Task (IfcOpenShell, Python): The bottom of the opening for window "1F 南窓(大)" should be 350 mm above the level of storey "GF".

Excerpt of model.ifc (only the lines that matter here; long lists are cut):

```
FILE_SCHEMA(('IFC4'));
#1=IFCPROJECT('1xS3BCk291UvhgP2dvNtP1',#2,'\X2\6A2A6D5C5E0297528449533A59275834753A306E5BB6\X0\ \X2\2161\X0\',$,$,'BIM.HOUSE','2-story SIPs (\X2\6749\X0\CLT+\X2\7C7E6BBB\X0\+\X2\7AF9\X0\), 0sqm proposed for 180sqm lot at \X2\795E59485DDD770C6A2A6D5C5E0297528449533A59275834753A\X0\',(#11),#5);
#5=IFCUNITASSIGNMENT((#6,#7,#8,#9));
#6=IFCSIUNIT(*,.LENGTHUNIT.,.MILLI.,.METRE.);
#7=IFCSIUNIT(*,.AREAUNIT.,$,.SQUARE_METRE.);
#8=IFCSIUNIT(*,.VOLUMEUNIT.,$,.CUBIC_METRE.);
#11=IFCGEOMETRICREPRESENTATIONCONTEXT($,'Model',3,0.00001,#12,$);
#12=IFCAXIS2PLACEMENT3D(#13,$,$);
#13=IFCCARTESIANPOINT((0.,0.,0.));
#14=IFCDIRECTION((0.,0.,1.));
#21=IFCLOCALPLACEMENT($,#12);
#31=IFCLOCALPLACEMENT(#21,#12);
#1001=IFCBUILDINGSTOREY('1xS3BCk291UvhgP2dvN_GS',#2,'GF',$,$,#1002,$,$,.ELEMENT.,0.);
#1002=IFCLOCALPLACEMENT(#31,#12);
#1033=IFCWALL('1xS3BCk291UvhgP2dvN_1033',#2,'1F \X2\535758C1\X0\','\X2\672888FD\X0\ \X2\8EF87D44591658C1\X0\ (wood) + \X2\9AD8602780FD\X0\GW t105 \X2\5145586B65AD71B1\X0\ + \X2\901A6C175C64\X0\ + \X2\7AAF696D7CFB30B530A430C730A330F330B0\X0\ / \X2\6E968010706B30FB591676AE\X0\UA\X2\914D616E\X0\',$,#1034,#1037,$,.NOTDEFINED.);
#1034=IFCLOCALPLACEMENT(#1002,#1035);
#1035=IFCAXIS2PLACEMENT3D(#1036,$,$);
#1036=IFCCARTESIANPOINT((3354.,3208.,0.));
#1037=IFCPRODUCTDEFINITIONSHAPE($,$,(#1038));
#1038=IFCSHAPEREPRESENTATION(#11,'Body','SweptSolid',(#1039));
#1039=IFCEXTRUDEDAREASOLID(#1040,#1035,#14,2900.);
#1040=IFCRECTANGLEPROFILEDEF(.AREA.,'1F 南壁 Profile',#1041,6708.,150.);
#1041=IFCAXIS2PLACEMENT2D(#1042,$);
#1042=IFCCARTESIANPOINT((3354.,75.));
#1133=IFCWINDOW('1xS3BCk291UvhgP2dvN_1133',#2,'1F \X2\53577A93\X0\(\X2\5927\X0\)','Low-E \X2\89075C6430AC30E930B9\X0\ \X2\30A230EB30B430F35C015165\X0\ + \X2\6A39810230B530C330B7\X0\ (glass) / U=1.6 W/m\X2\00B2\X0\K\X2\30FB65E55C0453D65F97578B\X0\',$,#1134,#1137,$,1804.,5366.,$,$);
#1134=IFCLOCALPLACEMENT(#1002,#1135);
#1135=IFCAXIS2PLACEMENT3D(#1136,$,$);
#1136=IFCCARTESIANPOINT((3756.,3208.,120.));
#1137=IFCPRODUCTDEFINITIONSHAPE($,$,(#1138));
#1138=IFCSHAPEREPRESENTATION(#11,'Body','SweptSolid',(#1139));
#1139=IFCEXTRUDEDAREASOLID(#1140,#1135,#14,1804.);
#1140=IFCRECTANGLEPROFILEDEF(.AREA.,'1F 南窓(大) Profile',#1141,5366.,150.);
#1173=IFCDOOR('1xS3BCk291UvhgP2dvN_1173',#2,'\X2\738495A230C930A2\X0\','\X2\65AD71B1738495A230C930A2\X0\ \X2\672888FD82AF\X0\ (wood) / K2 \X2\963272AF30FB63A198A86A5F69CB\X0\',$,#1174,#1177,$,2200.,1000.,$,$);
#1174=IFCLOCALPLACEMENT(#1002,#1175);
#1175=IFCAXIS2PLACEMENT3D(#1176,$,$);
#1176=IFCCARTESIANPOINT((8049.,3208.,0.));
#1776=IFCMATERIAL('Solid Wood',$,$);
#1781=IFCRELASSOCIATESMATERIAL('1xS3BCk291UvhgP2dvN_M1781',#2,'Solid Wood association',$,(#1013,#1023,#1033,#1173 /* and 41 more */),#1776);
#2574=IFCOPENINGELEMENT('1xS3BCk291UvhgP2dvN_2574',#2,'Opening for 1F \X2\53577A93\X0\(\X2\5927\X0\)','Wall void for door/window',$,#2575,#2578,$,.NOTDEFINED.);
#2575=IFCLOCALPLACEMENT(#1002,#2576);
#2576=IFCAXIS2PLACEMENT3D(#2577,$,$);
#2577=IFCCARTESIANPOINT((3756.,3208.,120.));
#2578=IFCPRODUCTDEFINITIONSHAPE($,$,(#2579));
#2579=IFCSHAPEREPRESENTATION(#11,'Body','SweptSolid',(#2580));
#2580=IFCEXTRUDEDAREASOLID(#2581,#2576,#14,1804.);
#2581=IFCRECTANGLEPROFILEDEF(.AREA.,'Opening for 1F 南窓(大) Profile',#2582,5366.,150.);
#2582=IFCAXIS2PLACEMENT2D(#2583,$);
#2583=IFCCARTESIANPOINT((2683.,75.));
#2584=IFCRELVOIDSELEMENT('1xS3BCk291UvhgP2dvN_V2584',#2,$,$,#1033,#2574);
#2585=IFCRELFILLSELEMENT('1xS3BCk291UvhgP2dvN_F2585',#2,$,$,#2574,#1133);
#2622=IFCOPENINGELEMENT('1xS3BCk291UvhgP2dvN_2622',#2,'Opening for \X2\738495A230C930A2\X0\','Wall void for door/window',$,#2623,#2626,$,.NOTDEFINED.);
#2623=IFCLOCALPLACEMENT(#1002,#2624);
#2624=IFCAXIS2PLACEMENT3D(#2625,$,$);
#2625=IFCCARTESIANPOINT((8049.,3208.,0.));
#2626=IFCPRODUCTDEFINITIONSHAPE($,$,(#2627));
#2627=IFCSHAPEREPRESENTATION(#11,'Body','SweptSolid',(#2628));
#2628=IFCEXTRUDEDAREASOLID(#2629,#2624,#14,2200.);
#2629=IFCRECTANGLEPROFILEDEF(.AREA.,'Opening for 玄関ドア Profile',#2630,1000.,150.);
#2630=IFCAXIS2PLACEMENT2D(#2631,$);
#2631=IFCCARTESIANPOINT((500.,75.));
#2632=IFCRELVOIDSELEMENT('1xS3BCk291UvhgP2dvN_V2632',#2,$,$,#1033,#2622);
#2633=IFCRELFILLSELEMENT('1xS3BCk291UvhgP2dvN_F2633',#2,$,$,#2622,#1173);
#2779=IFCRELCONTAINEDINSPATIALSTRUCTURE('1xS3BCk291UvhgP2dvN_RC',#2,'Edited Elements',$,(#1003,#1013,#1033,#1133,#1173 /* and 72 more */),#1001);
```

```python
import numpy as np
import ifcopenshell
import ifcopenshell.api.geometry
import ifcopenshell.geom
import ifcopenshell.util.element
import ifcopenshell.util.placement
import ifcopenshell.util.shape
import ifcopenshell.util.unit

model = ifcopenshell.open("model.ifc")
unit_scale = ifcopenshell.util.unit.calculate_unit_scale(model)

window = model.by_guid("1xS3BCk291UvhgP2dvN_1133")
opening = window.FillsVoids[0].RelatingOpeningElement
storey = ifcopenshell.util.element.get_container(window, ifc_class="IfcBuildingStorey")
level = ifcopenshell.util.placement.get_local_placement(storey.ObjectPlacement)[2, 3]

# The opening's origin need not be at the sill, so measure its lowest point.
shape = ifcopenshell.geom.create_shape(ifcopenshell.geom.settings(), opening)
bottom = ifcopenshell.util.shape.get_shape_bottom_elevation(shape, shape.geometry) / unit_scale
dz = level + 350.0 - bottom

shift = np.array([0.0, 0.0, dz])
# The window is not placed relative to its opening, so move both.
for product in (opening, window):
    matrix = ifcopenshell.util.placement.get_local_placement(product.ObjectPlacement)
    matrix[:3, 3] += shift
    ifcopenshell.api.geometry.edit_object_placement(model, product=product, matrix=matrix, is_si=False)

print(f"moved by {dz * unit_scale:+.3f} m")

model.write("model-out.ifc")
```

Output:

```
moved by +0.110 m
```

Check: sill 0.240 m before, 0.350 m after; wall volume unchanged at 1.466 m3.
